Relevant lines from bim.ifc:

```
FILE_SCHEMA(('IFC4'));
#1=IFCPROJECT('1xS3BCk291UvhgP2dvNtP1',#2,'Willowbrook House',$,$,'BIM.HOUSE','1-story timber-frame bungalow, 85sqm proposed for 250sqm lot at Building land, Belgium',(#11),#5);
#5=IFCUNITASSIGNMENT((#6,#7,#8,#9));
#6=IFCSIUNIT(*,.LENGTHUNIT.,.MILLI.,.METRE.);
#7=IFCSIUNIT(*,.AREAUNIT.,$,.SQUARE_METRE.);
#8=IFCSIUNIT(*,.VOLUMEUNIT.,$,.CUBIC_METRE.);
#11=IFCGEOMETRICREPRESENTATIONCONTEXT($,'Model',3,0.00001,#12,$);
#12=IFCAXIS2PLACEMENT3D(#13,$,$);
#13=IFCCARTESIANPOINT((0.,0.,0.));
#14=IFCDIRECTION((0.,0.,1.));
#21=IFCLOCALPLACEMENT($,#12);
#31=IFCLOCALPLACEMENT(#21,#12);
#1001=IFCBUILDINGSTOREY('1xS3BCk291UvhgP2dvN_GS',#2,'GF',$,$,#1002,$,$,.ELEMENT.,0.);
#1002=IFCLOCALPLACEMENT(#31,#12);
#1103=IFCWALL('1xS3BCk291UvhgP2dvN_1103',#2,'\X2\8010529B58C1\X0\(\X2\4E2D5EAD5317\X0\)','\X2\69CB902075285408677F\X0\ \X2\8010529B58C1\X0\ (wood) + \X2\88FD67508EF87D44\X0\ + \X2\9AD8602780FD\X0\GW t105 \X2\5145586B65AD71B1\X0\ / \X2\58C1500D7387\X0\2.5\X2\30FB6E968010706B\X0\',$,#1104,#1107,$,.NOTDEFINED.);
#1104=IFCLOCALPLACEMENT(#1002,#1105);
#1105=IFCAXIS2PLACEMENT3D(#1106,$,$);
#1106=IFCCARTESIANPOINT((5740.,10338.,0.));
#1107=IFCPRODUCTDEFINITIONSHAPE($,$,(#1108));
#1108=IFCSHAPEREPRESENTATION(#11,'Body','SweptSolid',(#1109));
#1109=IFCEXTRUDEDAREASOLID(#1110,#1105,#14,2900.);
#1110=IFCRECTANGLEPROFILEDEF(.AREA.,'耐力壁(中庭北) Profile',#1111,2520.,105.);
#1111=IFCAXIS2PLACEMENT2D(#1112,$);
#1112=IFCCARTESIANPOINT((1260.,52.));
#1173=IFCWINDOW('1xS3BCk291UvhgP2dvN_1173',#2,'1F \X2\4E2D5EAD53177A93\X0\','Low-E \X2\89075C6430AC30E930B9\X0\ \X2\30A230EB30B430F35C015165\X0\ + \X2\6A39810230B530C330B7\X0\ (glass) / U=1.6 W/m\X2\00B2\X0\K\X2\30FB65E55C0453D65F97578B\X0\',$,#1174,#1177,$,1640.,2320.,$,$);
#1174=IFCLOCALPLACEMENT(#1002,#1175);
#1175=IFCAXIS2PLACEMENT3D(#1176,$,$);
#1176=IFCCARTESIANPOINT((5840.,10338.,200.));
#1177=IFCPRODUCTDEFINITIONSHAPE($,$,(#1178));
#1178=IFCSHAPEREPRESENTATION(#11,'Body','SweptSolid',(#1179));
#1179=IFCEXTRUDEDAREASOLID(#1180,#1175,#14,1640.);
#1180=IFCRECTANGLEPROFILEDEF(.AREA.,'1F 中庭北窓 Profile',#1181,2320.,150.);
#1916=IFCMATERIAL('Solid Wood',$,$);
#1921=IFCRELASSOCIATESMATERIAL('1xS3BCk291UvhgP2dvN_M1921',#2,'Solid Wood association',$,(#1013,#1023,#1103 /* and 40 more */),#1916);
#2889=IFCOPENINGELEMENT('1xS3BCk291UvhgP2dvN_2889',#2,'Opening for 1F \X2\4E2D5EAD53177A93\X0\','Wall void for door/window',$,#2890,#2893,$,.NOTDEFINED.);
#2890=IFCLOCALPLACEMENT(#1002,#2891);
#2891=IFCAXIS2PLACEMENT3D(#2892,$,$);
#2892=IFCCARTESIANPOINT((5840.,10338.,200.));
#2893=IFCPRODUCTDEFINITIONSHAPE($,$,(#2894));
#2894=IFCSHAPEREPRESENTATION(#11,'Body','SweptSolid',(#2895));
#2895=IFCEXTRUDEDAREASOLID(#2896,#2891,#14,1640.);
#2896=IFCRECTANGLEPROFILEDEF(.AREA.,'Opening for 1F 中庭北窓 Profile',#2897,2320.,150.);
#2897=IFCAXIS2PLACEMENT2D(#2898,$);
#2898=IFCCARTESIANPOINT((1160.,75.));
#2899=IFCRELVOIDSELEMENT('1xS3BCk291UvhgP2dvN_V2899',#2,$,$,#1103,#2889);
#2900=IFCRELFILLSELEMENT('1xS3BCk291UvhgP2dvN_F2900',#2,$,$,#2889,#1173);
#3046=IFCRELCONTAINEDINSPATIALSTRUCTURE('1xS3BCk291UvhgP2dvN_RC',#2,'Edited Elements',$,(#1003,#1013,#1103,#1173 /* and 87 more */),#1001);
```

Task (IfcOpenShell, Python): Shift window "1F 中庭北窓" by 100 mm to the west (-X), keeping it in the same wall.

```python
import ifcopenshell
import ifcopenshell.api.geometry
import ifcopenshell.util.placement
import ifcopenshell.util.unit

model = ifcopenshell.open("bim.ifc")
unit_scale = ifcopenshell.util.unit.calculate_unit_scale(model)

window = model.by_id(1173)
opening = window.FillsVoids[0].RelatingOpeningElement
wall = opening.VoidsElements[0].RelatingBuildingElement

wall_matrix = ifcopenshell.util.placement.get_local_placement(wall.ObjectPlacement)
shift = wall_matrix[:3, 0] * -0.1 / unit_scale
before = ifcopenshell.util.placement.get_local_placement(window.ObjectPlacement)[:3, 3].copy()

# The window is not placed relative to its opening, so move both.
for product in (opening, window):
    matrix = ifcopenshell.util.placement.get_local_placement(product.ObjectPlacement)
    matrix[:3, 3] += shift
    ifcopenshell.api.geometry.edit_object_placement(model, product=product, matrix=matrix, is_si=False)

after = ifcopenshell.util.placement.get_local_placement(window.ObjectPlacement)[:3, 3]
print("window moved by", (after - before).round(3) + 0.0)

model.write("bim_updated.ifc")
```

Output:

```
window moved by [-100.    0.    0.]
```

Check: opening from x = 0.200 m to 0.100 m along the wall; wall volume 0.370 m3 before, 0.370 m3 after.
